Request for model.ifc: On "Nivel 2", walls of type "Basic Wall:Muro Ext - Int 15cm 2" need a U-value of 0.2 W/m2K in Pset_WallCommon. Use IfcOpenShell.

First a look at what the model holds.

```python
import ifcopenshell
import ifcopenshell.util.element

model = ifcopenshell.open("model.ifc")
print(model.schema)
storey = next(s for s in model.by_type("IfcBuildingStorey") if s.Name == "Nivel 2")
walls = [e for e in ifcopenshell.util.element.get_decomposition(storey) if e.is_a("IfcWall")]
seen = {}
for e in walls:
    element_type = ifcopenshell.util.element.get_type(e)
    key = (element_type.Name if element_type != e and element_type else None, ifcopenshell.util.element.get_pset(e, "Pset_WallCommon", "ThermalTransmittance"))
    seen[key] = seen.get(key, 0) + 1
for (name, value), count in sorted(seen.items(), key=str):
    print(count, "x", name, "|", value)
```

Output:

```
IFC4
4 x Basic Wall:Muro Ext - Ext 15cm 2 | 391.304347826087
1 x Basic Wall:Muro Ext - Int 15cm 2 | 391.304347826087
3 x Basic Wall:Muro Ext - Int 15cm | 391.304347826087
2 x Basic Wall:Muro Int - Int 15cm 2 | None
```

```python
import ifcopenshell
import ifcopenshell.api.pset
import ifcopenshell.util.element

model = ifcopenshell.open("model.ifc")

storey = next(s for s in model.by_type("IfcBuildingStorey") if s.Name == "Nivel 2")
walls = [e for e in ifcopenshell.util.element.get_decomposition(storey) if e.is_a("IfcWall")]

count = 0
for e in walls:
    element_type = ifcopenshell.util.element.get_type(e)
    if element_type in (None, e) or element_type.Name != "Basic Wall:Muro Ext - Int 15cm 2":
        continue
    # add_pset returns the element's existing set when there is one.
    pset = ifcopenshell.api.pset.add_pset(model, product=e, name="Pset_WallCommon")
    ifcopenshell.api.pset.edit_pset(model, pset=pset, properties={"ThermalTransmittance": 0.2})
    count += 1

print(count, "walls updated")

model.write("model_v2.ifc")
```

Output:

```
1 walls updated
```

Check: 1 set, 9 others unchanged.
